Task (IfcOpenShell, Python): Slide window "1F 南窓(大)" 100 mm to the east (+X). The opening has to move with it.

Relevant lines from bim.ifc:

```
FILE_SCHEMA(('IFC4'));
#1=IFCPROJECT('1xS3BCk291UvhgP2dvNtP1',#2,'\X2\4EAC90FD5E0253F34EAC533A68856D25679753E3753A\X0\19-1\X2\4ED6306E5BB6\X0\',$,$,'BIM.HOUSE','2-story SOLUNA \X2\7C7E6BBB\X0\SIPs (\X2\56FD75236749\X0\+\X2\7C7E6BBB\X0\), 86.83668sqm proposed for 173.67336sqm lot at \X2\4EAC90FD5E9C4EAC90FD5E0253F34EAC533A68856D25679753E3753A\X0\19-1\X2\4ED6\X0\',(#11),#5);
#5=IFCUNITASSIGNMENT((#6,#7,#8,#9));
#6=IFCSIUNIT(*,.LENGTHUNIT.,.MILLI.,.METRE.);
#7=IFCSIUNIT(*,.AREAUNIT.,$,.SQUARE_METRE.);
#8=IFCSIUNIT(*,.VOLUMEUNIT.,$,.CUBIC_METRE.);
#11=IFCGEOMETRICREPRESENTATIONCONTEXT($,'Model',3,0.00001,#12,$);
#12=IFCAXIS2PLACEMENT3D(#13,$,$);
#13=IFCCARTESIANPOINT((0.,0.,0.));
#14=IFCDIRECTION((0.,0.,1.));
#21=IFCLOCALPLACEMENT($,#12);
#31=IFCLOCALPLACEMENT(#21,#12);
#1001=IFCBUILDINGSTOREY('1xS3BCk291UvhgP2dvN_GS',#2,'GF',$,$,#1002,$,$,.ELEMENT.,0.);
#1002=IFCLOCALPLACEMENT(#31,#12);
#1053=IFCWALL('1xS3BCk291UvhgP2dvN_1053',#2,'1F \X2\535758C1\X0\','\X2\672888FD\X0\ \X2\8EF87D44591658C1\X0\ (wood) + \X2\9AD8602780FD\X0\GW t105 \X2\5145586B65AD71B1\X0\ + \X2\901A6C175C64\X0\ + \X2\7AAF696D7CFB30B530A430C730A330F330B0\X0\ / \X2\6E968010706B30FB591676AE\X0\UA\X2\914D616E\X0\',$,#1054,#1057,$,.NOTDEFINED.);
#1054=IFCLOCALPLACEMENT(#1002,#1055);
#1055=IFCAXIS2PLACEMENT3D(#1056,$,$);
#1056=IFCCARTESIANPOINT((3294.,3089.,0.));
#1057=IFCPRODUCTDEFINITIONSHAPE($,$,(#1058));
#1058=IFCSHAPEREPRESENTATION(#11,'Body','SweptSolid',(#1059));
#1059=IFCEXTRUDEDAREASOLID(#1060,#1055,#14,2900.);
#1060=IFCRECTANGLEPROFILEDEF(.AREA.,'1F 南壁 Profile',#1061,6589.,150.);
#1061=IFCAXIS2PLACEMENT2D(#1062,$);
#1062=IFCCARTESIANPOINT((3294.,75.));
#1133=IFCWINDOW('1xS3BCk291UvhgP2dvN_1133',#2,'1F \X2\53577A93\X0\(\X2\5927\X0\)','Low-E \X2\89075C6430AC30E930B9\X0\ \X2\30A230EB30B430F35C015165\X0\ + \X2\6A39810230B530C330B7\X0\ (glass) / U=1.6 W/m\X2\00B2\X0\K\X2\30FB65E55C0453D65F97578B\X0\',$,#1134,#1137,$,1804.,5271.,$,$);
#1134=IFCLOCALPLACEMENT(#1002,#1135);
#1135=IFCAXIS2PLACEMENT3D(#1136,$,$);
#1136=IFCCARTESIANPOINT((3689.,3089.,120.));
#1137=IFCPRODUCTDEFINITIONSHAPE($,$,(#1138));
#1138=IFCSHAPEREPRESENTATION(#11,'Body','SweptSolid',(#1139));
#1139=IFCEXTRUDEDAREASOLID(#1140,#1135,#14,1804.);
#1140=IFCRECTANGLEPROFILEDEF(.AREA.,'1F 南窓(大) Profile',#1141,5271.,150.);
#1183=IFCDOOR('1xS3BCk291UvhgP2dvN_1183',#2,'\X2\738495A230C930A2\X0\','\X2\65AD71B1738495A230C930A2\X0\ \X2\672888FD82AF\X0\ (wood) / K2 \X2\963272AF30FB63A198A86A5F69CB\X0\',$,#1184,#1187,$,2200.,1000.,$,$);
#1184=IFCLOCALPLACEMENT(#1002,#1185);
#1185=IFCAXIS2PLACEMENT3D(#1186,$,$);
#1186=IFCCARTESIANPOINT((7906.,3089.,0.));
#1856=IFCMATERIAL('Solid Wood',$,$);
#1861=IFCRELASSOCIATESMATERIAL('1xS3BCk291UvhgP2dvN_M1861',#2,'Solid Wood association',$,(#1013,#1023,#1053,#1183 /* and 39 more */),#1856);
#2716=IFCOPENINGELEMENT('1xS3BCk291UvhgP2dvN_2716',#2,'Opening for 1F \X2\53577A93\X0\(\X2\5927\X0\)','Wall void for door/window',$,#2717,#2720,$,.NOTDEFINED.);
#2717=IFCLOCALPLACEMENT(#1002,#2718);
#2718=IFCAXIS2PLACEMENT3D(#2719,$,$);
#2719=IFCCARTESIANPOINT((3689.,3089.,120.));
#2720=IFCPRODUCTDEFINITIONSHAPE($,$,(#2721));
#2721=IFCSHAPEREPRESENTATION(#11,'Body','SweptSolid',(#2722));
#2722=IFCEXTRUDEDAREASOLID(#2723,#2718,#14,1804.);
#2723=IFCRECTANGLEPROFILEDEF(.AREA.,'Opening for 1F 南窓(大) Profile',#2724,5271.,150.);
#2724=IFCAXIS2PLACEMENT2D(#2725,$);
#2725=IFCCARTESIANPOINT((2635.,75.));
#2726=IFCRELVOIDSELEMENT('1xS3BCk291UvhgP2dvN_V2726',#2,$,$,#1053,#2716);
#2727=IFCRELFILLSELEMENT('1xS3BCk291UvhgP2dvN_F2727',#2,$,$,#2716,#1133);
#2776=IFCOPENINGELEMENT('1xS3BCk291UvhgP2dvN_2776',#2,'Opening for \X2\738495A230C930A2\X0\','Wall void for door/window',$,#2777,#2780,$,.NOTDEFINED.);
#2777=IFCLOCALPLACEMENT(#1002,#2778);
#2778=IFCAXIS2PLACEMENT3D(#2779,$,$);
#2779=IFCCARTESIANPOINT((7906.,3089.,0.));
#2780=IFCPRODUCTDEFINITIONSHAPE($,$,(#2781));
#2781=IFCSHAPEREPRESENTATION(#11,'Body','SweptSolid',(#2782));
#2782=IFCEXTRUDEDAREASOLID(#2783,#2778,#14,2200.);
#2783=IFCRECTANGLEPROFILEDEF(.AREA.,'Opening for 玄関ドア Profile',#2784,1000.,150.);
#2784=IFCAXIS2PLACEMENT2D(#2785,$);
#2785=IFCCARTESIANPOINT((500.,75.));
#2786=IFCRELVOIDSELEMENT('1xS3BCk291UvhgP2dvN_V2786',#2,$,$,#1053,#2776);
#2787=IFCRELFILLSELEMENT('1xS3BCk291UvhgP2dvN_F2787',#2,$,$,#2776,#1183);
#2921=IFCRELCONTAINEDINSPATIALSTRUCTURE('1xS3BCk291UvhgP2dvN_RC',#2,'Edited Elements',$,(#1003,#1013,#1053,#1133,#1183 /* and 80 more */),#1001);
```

```python
import ifcopenshell
import ifcopenshell.api.geometry
import ifcopenshell.util.placement

model = ifcopenshell.open("bim.ifc")

window = model.by_guid("1xS3BCk291UvhgP2dvN_1133")
opening = window.FillsVoids[0].RelatingOpeningElement
wall = opening.VoidsElements[0].RelatingBuildingElement

wall_matrix = ifcopenshell.util.placement.get_local_placement(wall.ObjectPlacement)
shift = wall_matrix[:3, 0] * 100.0
before = ifcopenshell.util.placement.get_local_placement(window.ObjectPlacement)[:3, 3].copy()

# The window is not placed relative to its opening, so move both.
for product in (opening, window):
    matrix = ifcopenshell.util.placement.get_local_placement(product.ObjectPlacement)
    matrix[:3, 3] += shift
    ifcopenshell.api.geometry.edit_object_placement(model, product=product, matrix=matrix, is_si=False)

after = ifcopenshell.util.placement.get_local_placement(window.ObjectPlacement)[:3, 3]
print("window moved by", (after - before).round(3) + 0.0)

model.write("bim-out.ifc")
```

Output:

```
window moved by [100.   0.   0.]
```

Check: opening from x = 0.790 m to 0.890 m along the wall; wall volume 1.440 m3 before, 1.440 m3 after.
